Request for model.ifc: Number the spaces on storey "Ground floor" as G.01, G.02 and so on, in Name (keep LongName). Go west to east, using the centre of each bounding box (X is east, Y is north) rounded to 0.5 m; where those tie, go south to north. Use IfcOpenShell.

First a look at what the model holds.

```python
import ifcopenshell
import ifcopenshell.util.element
import ifcopenshell.util.placement

model = ifcopenshell.open("model.ifc")
print(model.schema)
storey = next(s for s in model.by_type("IfcBuildingStorey") if s.Name == "Ground floor")
spaces = [e for e in ifcopenshell.util.element.get_decomposition(storey) if e.is_a("IfcSpace")]
for e in sorted(spaces, key=lambda e: e.id()):
    origin = ifcopenshell.util.placement.get_local_placement(e.ObjectPlacement)[:3, 3]
    print(e.id(), e.Name, e.LongName, origin.round(2) + 0.0, sep=" | ")
```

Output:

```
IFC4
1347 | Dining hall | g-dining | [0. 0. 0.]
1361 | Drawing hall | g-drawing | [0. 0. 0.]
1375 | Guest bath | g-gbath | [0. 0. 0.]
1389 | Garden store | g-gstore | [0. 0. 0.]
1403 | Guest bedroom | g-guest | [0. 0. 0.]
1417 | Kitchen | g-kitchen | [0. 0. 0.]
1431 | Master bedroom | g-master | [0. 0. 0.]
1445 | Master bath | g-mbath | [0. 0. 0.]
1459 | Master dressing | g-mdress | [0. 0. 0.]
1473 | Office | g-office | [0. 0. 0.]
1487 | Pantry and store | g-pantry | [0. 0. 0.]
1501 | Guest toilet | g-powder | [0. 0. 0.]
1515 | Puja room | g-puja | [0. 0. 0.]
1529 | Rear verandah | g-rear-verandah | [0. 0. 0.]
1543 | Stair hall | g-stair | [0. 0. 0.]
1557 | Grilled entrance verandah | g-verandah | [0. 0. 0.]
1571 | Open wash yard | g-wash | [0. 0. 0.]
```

```python
import ifcopenshell
import ifcopenshell.geom
import ifcopenshell.util.element
import ifcopenshell.util.shape

model = ifcopenshell.open("model.ifc")
settings = ifcopenshell.geom.settings()
settings.set("use-world-coords", True)


def centre(element):
    shape = ifcopenshell.geom.create_shape(settings, element)
    return ifcopenshell.util.shape.get_bbox_centroid(shape.geometry)


storey = next(s for s in model.by_type("IfcBuildingStorey") if s.Name == "Ground floor")
spaces = [e for e in ifcopenshell.util.element.get_decomposition(storey) if e.is_a("IfcSpace")]

# Insertion points can sit at a corner or the storey origin, so sort by the geometry (in metres).
centres = {e: centre(e) for e in spaces}
spaces.sort(key=lambda e: (round(centres[e][0] / 0.5), centres[e][1]))

for i, e in enumerate(spaces, start=1):
    number = f"G.{i:02d}"
    e.Name = number
    print(e.id(), number)

model.write("model_rev.ifc")
```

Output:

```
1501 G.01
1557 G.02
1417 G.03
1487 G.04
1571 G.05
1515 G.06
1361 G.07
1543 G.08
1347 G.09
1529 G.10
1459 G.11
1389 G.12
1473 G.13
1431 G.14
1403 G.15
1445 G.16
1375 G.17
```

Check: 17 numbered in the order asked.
